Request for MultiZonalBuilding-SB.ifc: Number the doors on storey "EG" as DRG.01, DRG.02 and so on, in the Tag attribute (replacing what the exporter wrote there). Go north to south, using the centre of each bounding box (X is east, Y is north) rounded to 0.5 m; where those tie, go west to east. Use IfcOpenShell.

First a look at what the model holds.

```python
import ifcopenshell
import ifcopenshell.util.element
import ifcopenshell.util.placement

model = ifcopenshell.open("MultiZonalBuilding-SB.ifc")
print(model.schema)
storey = next(s for s in model.by_type("IfcBuildingStorey") if s.Name == "EG")
doors = [e for e in ifcopenshell.util.element.get_decomposition(storey) if e.is_a("IfcDoor")]
for e in sorted(doors, key=lambda e: e.id()):
    origin = ifcopenshell.util.placement.get_local_placement(e.ObjectPlacement)[:3, 3]
    print(e.id(), e.Tag, e.Name, origin.round(2) + 0.0, sep=" | ")
```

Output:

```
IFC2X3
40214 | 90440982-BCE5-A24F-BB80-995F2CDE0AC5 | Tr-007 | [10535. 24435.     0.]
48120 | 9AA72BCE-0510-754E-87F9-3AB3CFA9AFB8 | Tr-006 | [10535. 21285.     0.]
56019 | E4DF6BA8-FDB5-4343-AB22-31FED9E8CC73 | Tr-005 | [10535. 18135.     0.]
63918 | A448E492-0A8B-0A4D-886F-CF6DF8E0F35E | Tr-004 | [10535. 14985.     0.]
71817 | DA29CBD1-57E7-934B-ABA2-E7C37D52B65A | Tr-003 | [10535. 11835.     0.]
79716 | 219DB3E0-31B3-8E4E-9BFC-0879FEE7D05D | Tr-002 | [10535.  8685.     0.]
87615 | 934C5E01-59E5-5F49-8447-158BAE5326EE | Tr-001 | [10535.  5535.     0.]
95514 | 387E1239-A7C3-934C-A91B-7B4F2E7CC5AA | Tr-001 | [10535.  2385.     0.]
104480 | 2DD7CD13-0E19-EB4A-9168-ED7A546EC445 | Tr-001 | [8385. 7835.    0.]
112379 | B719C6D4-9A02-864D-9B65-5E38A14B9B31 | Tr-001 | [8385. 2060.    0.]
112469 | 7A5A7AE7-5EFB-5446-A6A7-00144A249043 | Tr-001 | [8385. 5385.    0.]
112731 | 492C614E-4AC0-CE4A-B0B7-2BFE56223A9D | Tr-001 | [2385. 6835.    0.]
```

```python
import ifcopenshell
import ifcopenshell.geom
import ifcopenshell.util.element
import ifcopenshell.util.shape

model = ifcopenshell.open("MultiZonalBuilding-SB.ifc")
settings = ifcopenshell.geom.settings()
settings.set("use-world-coords", True)


def centre(element):
    shape = ifcopenshell.geom.create_shape(settings, element)
    return ifcopenshell.util.shape.get_bbox_centroid(shape.geometry)


storey = next(s for s in model.by_type("IfcBuildingStorey") if s.Name == "EG")
doors = [e for e in ifcopenshell.util.element.get_decomposition(storey) if e.is_a("IfcDoor")]

# Insertion points can sit at a corner or the storey origin, so sort by the geometry (in metres).
centres = {e: centre(e) for e in doors}
doors.sort(key=lambda e: (-round(centres[e][1] / 0.5), centres[e][0]))

for i, e in enumerate(doors, start=1):
    number = f"DRG.{i:02d}"
    e.Tag = number
    print(e.id(), number)

model.write("MultiZonalBuilding-SB-out.ifc")
```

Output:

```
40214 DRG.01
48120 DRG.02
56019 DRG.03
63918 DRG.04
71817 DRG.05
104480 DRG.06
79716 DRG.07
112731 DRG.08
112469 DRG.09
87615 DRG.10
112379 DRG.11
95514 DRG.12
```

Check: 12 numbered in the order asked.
